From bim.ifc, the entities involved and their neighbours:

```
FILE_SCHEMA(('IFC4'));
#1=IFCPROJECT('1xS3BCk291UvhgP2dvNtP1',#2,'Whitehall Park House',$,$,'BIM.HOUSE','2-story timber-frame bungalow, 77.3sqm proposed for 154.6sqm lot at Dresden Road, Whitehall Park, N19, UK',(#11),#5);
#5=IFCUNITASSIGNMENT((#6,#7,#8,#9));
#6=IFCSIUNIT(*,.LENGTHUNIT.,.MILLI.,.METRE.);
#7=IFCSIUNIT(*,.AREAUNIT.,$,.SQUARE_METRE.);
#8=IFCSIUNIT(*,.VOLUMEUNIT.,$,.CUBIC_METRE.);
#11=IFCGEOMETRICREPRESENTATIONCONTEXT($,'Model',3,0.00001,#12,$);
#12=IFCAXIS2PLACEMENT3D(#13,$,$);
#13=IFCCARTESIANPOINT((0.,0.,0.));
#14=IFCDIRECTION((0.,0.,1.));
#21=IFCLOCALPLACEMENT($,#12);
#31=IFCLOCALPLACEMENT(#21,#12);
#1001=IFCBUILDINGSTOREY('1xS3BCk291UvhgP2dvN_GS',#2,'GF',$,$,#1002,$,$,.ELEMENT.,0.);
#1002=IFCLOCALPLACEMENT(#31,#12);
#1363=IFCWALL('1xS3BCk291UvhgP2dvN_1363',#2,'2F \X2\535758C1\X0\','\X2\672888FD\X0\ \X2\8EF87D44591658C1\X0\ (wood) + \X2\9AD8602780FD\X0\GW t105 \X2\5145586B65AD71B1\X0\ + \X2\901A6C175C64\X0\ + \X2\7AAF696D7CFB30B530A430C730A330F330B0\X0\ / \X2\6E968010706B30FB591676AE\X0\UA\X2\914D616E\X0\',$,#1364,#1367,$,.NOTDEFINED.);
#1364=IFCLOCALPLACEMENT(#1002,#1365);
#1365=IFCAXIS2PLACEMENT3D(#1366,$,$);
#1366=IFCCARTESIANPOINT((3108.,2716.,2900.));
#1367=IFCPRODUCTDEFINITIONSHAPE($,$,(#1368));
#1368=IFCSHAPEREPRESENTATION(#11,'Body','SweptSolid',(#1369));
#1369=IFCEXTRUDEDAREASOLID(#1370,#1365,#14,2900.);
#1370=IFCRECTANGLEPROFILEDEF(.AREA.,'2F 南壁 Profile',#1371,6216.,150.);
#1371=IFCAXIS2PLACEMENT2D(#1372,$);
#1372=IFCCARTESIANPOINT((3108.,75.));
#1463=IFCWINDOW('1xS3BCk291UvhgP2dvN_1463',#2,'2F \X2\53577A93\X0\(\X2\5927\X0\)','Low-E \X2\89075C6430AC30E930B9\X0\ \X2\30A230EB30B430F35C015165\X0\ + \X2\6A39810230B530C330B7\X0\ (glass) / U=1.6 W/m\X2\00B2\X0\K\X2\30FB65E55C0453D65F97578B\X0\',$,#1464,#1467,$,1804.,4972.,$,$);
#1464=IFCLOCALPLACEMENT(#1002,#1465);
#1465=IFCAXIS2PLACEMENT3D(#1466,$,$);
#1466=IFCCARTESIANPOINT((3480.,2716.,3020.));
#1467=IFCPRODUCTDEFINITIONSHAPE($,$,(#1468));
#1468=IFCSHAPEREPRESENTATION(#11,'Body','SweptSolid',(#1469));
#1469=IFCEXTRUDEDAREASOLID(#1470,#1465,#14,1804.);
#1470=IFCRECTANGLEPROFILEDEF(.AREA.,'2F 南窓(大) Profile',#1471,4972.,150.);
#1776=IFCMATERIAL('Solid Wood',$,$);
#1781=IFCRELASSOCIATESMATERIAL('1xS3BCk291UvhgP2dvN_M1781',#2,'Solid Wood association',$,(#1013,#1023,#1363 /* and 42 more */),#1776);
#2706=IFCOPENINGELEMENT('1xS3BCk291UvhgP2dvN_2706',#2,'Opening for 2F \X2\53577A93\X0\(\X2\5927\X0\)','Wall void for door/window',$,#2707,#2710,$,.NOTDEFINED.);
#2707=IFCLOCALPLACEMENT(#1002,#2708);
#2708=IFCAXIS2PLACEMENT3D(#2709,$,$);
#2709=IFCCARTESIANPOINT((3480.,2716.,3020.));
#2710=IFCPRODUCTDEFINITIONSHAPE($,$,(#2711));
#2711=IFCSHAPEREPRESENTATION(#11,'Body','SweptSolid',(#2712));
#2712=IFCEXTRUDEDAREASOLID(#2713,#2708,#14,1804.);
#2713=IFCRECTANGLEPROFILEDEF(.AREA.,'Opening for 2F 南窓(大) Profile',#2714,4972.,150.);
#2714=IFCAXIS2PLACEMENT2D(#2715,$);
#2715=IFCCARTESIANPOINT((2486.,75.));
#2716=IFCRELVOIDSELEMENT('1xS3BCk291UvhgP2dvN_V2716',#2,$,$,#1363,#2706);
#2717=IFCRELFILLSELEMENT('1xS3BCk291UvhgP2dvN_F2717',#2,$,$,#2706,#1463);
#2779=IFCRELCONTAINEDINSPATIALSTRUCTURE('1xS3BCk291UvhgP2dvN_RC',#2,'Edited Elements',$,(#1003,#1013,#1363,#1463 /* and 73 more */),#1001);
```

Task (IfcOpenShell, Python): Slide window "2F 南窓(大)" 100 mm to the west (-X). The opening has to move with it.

```python
import ifcopenshell
import ifcopenshell.api.geometry
import ifcopenshell.util.placement
import ifcopenshell.util.unit

model = ifcopenshell.open("bim.ifc")
unit_scale = ifcopenshell.util.unit.calculate_unit_scale(model)

window = model.by_guid("1xS3BCk291UvhgP2dvN_1463")
opening = window.FillsVoids[0].RelatingOpeningElement
wall = opening.VoidsElements[0].RelatingBuildingElement

wall_matrix = ifcopenshell.util.placement.get_local_placement(wall.ObjectPlacement)
shift = wall_matrix[:3, 0] * -0.1 / unit_scale
before = ifcopenshell.util.placement.get_local_placement(window.ObjectPlacement)[:3, 3].copy()

# The window is not placed relative to its opening, so move both.
for product in (opening, window):
    matrix = ifcopenshell.util.placement.get_local_placement(product.ObjectPlacement)
    matrix[:3, 3] += shift
    ifcopenshell.api.geometry.edit_object_placement(model, product=product, matrix=matrix, is_si=False)

after = ifcopenshell.util.placement.get_local_placement(window.ObjectPlacement)[:3, 3]
print("window moved by", (after - before).round(3) + 0.0)

model.write("bim_v2.ifc")
```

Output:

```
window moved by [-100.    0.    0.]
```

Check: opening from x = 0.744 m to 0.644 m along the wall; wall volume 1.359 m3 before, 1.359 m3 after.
